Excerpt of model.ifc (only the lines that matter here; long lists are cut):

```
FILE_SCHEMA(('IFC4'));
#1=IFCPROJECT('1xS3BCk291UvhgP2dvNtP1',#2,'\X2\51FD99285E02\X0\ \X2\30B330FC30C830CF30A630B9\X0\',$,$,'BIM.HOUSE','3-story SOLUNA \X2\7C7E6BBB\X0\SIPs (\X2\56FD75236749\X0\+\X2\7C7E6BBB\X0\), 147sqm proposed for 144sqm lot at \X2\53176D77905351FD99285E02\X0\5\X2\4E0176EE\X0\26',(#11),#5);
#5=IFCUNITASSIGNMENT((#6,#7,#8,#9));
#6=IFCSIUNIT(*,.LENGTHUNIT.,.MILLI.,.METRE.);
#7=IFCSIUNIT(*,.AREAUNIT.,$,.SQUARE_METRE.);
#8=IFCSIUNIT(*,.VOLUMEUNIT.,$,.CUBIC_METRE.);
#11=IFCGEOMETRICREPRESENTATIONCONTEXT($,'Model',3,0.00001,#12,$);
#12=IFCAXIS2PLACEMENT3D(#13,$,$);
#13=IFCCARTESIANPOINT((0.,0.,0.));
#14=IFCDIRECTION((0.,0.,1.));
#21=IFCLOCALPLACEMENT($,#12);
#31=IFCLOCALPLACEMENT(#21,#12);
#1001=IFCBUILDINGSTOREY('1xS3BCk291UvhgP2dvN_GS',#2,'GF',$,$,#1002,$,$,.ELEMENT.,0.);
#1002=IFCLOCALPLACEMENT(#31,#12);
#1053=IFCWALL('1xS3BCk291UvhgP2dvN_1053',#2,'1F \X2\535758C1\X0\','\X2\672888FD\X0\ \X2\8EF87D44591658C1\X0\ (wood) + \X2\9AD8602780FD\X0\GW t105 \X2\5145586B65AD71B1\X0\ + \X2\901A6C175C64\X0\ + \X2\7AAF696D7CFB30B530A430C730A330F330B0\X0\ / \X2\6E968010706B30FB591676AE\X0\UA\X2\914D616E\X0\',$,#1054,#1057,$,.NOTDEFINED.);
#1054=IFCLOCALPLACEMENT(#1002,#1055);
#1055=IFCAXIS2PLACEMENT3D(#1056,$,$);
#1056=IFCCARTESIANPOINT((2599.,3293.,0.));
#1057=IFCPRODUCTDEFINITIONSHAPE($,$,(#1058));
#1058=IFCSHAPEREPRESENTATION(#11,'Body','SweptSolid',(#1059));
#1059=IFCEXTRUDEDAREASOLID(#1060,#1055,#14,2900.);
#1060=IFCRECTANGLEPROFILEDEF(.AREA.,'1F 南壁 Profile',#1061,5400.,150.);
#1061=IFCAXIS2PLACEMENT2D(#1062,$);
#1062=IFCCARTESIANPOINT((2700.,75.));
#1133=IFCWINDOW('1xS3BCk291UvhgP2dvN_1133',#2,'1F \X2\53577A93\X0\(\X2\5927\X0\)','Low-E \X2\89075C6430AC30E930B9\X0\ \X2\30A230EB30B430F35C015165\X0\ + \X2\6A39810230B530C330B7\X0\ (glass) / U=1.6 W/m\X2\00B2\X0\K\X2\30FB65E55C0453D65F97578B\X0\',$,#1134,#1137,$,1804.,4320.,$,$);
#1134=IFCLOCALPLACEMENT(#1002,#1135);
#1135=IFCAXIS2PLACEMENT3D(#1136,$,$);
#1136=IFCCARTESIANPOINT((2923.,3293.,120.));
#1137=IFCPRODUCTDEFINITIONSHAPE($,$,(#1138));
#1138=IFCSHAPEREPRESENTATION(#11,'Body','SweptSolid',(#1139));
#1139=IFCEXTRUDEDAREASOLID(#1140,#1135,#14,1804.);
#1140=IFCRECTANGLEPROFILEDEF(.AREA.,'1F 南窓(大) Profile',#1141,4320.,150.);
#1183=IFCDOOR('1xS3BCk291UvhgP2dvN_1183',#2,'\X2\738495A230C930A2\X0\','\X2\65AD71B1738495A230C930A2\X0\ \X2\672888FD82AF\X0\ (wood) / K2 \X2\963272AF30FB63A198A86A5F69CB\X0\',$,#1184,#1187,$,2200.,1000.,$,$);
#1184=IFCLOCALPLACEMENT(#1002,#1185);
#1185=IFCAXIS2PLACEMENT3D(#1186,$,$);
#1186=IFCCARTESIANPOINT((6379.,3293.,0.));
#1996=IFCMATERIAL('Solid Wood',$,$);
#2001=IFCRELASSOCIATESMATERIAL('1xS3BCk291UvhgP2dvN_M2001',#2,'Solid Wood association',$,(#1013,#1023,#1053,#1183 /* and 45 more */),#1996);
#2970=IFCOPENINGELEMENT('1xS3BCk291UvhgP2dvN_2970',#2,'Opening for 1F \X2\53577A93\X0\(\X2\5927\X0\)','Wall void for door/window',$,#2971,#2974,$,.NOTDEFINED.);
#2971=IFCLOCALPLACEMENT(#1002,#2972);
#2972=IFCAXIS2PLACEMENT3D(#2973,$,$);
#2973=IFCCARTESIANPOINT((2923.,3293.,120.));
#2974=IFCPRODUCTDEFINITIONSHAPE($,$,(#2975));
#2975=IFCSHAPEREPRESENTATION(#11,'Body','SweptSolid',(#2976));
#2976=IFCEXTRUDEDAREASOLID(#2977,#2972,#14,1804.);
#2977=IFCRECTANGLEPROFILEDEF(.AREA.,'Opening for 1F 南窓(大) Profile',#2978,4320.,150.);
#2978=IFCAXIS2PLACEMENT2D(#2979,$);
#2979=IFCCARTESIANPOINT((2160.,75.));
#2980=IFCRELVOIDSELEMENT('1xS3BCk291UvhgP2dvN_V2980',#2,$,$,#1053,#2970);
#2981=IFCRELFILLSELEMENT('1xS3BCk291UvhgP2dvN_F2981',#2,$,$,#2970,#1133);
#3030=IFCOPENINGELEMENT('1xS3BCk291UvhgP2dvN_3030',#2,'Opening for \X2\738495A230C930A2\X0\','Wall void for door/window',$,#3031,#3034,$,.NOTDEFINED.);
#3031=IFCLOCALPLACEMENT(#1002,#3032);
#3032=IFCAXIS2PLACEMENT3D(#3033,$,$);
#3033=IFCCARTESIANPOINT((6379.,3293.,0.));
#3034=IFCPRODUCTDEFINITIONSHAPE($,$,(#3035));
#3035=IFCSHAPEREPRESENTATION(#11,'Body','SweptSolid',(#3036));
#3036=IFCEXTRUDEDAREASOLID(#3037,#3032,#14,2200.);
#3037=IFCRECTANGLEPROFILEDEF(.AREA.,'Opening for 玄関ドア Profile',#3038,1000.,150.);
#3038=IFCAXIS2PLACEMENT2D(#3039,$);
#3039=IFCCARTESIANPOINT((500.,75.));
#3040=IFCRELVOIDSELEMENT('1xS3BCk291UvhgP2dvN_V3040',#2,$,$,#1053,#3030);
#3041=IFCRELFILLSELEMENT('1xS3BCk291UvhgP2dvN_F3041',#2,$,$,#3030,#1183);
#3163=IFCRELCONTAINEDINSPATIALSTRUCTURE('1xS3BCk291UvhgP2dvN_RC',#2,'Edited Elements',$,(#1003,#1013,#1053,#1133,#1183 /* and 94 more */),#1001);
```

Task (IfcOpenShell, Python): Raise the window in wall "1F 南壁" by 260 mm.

```python
import numpy as np
import ifcopenshell
import ifcopenshell.api.geometry
import ifcopenshell.util.placement
import ifcopenshell.util.unit

model = ifcopenshell.open("model.ifc")
unit_scale = ifcopenshell.util.unit.calculate_unit_scale(model)

window = model.by_guid("1xS3BCk291UvhgP2dvN_1133")
opening = window.FillsVoids[0].RelatingOpeningElement
dz = 260.0

shift = np.array([0.0, 0.0, dz])
# The window is not placed relative to its opening, so move both.
for product in (opening, window):
    matrix = ifcopenshell.util.placement.get_local_placement(product.ObjectPlacement)
    matrix[:3, 3] += shift
    ifcopenshell.api.geometry.edit_object_placement(model, product=product, matrix=matrix, is_si=False)

print(f"moved by {dz * unit_scale:+.3f} m")

model.write("model_edited.ifc")
```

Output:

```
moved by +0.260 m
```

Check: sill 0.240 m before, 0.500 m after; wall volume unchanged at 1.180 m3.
